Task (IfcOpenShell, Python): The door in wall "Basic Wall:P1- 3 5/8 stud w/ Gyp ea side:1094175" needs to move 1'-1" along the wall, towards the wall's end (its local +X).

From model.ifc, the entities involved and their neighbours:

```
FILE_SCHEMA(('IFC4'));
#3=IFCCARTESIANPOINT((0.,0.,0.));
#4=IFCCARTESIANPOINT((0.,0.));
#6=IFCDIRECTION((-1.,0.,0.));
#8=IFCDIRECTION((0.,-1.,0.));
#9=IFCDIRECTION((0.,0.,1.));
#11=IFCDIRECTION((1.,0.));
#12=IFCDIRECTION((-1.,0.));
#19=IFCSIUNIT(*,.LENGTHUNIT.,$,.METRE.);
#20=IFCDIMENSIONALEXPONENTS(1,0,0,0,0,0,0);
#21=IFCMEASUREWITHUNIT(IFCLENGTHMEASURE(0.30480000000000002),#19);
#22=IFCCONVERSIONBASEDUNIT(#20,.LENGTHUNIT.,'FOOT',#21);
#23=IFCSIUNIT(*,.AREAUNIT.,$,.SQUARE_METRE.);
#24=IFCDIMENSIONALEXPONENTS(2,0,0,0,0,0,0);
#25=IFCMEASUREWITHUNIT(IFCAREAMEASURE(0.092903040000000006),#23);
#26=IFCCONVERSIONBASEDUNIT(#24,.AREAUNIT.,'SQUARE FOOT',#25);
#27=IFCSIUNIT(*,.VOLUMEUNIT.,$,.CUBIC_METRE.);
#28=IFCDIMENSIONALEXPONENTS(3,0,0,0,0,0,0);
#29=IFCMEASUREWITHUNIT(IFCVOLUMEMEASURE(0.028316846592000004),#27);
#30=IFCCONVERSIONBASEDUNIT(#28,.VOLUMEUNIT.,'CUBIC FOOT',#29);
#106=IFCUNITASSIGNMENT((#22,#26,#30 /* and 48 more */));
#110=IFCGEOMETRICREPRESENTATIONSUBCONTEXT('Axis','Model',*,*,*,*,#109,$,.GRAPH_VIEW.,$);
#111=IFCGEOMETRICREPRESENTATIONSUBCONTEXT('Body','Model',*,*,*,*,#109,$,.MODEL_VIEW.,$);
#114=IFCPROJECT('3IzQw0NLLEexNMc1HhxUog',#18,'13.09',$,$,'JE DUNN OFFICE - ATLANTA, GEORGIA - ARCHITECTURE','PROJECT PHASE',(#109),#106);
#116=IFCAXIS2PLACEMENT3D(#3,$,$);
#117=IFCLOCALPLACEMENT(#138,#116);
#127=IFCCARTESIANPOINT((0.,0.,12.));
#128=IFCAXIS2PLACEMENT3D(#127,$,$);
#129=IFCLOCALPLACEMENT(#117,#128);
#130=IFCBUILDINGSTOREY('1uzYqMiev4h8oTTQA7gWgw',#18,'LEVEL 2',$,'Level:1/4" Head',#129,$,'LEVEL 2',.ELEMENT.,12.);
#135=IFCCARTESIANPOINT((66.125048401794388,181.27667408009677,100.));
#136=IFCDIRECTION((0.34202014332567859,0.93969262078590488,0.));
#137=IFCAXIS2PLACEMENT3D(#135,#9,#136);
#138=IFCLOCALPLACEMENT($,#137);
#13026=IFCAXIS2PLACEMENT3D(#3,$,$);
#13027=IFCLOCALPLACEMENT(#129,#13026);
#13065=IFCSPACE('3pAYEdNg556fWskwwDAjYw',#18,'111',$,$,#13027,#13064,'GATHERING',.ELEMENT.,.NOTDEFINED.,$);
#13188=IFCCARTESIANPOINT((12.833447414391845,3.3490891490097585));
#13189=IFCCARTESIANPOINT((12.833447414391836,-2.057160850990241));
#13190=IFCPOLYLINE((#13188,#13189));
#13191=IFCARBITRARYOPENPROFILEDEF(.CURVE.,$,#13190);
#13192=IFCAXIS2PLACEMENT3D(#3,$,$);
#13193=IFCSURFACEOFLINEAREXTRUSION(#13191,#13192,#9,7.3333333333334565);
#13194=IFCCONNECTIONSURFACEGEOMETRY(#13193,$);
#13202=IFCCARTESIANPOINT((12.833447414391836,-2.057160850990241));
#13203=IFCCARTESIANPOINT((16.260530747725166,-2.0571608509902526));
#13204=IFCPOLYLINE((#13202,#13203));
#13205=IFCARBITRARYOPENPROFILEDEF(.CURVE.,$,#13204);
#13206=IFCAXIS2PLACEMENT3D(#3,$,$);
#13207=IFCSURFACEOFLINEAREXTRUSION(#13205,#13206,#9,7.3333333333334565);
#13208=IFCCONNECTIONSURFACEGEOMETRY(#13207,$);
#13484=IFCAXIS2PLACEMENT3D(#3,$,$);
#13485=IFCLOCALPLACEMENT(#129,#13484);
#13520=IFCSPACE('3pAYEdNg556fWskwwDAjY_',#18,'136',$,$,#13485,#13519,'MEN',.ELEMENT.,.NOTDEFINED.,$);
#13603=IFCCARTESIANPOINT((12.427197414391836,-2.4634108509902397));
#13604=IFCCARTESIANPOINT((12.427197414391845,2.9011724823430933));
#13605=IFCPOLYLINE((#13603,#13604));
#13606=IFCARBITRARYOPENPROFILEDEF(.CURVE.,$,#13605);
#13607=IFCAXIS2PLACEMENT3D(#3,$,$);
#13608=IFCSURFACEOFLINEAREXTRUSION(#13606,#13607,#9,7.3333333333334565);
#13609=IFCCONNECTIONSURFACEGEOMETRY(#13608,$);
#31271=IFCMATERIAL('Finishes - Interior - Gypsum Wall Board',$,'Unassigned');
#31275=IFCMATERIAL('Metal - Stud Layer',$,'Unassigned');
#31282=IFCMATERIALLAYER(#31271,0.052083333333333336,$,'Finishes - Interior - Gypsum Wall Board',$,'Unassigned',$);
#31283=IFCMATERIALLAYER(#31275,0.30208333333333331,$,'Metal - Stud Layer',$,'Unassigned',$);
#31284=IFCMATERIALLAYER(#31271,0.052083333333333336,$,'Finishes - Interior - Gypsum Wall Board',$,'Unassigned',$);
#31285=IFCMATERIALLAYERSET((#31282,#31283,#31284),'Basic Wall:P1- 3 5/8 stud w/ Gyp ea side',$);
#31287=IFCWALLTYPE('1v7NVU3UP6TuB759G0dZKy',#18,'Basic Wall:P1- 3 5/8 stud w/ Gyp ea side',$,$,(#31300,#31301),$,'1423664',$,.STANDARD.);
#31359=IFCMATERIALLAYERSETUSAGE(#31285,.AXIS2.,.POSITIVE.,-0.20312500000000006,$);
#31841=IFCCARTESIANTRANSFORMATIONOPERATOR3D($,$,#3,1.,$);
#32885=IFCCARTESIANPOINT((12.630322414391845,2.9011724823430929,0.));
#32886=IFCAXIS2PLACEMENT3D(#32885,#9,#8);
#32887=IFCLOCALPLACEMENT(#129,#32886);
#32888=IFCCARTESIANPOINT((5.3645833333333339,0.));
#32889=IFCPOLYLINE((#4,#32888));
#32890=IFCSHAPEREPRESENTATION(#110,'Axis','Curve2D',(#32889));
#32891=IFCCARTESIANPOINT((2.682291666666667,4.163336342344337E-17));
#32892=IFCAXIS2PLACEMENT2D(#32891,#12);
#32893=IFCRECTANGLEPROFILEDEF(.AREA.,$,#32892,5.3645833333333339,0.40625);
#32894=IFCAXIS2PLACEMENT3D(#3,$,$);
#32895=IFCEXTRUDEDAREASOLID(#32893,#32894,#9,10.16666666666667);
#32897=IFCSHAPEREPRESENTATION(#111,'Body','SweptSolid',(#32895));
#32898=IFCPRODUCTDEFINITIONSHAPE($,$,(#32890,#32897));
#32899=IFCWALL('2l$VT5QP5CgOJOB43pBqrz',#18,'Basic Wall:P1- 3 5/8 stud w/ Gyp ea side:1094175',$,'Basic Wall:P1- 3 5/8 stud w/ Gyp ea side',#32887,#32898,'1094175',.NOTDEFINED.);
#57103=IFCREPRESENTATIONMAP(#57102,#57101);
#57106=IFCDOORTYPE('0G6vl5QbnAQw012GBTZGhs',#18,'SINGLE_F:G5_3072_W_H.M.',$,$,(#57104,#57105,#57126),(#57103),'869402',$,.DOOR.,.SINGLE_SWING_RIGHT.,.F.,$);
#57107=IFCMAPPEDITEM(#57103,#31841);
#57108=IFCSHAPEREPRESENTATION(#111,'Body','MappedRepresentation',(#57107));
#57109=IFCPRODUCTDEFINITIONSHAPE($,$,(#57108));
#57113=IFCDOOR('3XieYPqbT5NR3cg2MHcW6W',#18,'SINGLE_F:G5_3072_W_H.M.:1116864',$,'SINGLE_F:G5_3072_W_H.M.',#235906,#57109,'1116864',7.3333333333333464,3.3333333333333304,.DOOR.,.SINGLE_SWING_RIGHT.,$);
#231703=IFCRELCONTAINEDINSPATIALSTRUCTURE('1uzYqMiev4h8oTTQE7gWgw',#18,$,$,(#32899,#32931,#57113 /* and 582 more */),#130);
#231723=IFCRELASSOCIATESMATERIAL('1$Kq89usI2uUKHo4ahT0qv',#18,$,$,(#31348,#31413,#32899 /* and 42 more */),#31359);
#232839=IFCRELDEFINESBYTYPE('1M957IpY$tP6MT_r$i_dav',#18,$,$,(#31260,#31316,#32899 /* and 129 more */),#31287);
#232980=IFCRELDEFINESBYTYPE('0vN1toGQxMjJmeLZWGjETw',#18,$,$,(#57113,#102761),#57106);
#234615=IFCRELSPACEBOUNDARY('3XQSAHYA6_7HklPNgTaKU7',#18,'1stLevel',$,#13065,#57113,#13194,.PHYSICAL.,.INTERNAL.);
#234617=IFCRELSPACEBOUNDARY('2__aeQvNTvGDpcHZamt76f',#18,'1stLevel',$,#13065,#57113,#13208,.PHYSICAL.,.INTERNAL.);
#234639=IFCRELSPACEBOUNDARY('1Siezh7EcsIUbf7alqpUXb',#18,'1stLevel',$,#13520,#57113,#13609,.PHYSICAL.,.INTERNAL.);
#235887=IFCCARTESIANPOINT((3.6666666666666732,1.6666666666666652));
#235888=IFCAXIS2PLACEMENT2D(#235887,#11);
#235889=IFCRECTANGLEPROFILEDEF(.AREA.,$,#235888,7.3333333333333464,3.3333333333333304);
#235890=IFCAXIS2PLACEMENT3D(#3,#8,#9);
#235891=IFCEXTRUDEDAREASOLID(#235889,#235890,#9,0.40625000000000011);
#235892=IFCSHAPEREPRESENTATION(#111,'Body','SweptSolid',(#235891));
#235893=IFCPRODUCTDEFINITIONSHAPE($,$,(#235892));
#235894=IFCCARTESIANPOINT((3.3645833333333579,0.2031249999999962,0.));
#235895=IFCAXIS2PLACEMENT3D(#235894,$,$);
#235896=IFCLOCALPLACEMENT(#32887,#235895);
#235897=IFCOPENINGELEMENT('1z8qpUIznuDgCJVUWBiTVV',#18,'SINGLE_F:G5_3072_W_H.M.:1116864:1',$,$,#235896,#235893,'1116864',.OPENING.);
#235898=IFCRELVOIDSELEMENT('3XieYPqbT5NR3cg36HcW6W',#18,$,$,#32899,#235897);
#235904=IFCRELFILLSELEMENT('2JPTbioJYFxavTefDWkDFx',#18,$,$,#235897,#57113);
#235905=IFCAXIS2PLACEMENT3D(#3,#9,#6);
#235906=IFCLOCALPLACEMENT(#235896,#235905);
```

```python
import numpy as np
import ifcopenshell
import ifcopenshell.api.geometry
import ifcopenshell.util.placement
import ifcopenshell.util.unit

model = ifcopenshell.open("model.ifc")
unit_scale = ifcopenshell.util.unit.calculate_unit_scale(model)

door = model.by_guid("3XieYPqbT5NR3cg2MHcW6W")
opening = door.FillsVoids[0].RelatingOpeningElement
wall = opening.VoidsElements[0].RelatingBuildingElement

wall_matrix = ifcopenshell.util.placement.get_local_placement(wall.ObjectPlacement)
shift = wall_matrix[:3, 0] * 13 * 0.0254 / unit_scale
before = ifcopenshell.util.placement.get_local_placement(door.ObjectPlacement)[:3, 3].copy()

# The door is placed relative to its opening, so it follows when the opening moves.
matrix = ifcopenshell.util.placement.get_local_placement(opening.ObjectPlacement)
matrix[:3, 3] += shift
ifcopenshell.api.geometry.edit_object_placement(
    model, product=opening, matrix=matrix, is_si=False, should_transform_children=True
)

# Space boundary surfaces are stored in each space's coordinates; move them too.
for rel in door.ProvidesBoundaries:
    if not rel.ConnectionGeometry:
        continue
    surface = rel.ConnectionGeometry.SurfaceOnRelatingElement
    space_matrix = ifcopenshell.util.placement.get_local_placement(rel.RelatingSpace.ObjectPlacement)
    point = np.array(surface.Position.Location.Coordinates) + space_matrix[:3, :3].T @ shift
    surface.Position = model.createIfcAxis2Placement3D(
        model.createIfcCartesianPoint(point.tolist()), surface.Position.Axis, surface.Position.RefDirection
    )

after = ifcopenshell.util.placement.get_local_placement(door.ObjectPlacement)[:3, 3]
print("door moved by", (after - before).round(3) + 0.0)

model.write("model_v2.ifc")
```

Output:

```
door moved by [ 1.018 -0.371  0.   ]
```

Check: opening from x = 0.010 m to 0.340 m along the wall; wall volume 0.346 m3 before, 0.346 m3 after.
